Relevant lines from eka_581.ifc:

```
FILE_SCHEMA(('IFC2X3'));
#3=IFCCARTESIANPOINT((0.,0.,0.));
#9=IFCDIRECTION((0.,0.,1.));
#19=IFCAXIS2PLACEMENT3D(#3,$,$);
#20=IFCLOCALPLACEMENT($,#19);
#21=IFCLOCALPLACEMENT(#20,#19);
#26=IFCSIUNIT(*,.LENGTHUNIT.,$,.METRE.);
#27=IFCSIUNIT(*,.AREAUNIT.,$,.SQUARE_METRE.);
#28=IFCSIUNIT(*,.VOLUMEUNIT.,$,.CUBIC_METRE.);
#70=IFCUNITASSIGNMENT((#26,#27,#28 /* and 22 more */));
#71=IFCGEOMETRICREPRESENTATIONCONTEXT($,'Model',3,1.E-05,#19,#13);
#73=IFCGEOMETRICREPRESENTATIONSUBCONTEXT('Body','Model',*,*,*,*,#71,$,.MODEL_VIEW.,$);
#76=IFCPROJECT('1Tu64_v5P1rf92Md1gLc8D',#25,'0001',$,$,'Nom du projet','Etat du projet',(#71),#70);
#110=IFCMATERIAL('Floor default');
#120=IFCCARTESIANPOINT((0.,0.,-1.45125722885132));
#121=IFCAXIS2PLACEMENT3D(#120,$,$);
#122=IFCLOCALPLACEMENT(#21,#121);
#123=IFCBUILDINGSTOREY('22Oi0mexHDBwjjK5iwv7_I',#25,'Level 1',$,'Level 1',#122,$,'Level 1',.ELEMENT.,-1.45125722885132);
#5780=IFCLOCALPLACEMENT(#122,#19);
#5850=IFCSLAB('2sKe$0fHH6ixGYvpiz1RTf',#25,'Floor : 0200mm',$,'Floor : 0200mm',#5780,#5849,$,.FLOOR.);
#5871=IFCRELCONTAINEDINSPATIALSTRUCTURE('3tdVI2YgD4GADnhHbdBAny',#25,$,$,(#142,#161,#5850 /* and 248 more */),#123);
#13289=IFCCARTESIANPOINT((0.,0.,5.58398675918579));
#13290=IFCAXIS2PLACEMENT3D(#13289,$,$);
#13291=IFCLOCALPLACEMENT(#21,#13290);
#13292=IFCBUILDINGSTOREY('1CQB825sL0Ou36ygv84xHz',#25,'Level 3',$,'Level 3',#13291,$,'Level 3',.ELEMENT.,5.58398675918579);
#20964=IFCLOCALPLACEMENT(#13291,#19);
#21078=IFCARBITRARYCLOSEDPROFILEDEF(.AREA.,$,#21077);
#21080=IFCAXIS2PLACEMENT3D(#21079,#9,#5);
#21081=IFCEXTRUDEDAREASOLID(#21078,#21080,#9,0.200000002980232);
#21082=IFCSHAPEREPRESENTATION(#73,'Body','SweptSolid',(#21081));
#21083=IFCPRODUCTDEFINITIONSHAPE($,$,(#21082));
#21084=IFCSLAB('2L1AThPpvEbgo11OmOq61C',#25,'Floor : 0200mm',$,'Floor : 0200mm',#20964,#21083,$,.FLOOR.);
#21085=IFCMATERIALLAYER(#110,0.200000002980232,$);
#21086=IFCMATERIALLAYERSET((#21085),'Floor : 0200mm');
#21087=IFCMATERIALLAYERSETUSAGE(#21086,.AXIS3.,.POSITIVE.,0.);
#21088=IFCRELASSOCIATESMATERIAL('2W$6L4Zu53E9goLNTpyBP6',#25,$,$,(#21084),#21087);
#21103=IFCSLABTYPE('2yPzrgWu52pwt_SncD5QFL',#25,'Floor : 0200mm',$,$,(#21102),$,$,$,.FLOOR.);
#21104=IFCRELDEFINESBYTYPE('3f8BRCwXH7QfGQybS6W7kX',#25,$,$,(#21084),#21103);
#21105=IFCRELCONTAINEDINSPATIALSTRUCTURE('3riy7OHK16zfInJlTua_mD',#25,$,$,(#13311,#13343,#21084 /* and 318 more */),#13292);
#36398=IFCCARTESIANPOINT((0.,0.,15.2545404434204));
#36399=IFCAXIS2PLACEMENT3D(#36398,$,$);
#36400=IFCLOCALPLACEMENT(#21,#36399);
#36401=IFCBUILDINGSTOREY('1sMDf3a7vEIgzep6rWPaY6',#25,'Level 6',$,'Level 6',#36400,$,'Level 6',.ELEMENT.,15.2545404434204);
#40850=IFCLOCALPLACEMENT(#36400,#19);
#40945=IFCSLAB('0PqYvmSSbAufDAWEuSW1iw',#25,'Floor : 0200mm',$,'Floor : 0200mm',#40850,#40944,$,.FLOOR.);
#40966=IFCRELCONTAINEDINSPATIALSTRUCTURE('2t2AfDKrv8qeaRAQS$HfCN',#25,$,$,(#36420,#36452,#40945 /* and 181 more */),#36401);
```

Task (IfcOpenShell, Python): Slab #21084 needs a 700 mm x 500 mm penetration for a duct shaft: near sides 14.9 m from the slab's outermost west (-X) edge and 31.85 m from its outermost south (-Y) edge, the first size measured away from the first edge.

```python
import numpy as np
import ifcopenshell
import ifcopenshell.api.feature
import ifcopenshell.api.geometry
import ifcopenshell.api.root
import ifcopenshell.geom
import ifcopenshell.util.placement
import ifcopenshell.util.representation
import ifcopenshell.util.shape
import ifcopenshell.util.unit

model = ifcopenshell.open("eka_581.ifc")
unit_scale = ifcopenshell.util.unit.calculate_unit_scale(model)
settings = ifcopenshell.geom.settings()


def volume(element):
    """Net volume in cubic metres, openings subtracted."""
    shape = ifcopenshell.geom.create_shape(settings, element)
    return ifcopenshell.util.shape.get_volume(shape.geometry)


slab = model.by_guid("2L1AThPpvEbgo11OmOq61C")
before = volume(slab)

# Extent in the slab's own axes, in metres. The edges named are its -X and -Y sides.
slab_shape = ifcopenshell.geom.create_shape(settings, slab)
vertices = ifcopenshell.util.shape.get_vertices(slab_shape.geometry)
x_min, y_min, bottom = vertices.min(axis=0)
top = vertices[:, 2].max()

opening = ifcopenshell.api.root.create_entity(model, ifc_class="IfcOpeningElement", name="Duct shaft opening")
context = ifcopenshell.util.representation.get_context(model, "Model", "Body", "MODEL_VIEW")
width, depth = 0.7, 0.5
outline = [(0.0, 0.0), (width, 0.0), (width, depth), (0.0, depth), (0.0, 0.0)]
# Overshoot both faces by 50 mm so the cut is clean.
shape = ifcopenshell.api.geometry.add_slab_representation(
    model, context=context, depth=top - bottom + 0.1, polyline=outline
)
ifcopenshell.api.geometry.assign_representation(model, product=opening, representation=shape)

matrix = ifcopenshell.util.placement.get_local_placement(slab.ObjectPlacement)
matrix[:, 3] = matrix @ np.append(np.array([x_min + 14.9, y_min + 31.85, bottom - 0.05]) / unit_scale, 1.0)
ifcopenshell.api.geometry.edit_object_placement(model, product=opening, matrix=matrix, is_si=False)
ifcopenshell.api.feature.add_feature(model, feature=opening, element=slab)

after = volume(slab)

print(f"slab volume {before:.3f} -> {after:.3f} m3")

model.write("eka_581_edited.ifc")
```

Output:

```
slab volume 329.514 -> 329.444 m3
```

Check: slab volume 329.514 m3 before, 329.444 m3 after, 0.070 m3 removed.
